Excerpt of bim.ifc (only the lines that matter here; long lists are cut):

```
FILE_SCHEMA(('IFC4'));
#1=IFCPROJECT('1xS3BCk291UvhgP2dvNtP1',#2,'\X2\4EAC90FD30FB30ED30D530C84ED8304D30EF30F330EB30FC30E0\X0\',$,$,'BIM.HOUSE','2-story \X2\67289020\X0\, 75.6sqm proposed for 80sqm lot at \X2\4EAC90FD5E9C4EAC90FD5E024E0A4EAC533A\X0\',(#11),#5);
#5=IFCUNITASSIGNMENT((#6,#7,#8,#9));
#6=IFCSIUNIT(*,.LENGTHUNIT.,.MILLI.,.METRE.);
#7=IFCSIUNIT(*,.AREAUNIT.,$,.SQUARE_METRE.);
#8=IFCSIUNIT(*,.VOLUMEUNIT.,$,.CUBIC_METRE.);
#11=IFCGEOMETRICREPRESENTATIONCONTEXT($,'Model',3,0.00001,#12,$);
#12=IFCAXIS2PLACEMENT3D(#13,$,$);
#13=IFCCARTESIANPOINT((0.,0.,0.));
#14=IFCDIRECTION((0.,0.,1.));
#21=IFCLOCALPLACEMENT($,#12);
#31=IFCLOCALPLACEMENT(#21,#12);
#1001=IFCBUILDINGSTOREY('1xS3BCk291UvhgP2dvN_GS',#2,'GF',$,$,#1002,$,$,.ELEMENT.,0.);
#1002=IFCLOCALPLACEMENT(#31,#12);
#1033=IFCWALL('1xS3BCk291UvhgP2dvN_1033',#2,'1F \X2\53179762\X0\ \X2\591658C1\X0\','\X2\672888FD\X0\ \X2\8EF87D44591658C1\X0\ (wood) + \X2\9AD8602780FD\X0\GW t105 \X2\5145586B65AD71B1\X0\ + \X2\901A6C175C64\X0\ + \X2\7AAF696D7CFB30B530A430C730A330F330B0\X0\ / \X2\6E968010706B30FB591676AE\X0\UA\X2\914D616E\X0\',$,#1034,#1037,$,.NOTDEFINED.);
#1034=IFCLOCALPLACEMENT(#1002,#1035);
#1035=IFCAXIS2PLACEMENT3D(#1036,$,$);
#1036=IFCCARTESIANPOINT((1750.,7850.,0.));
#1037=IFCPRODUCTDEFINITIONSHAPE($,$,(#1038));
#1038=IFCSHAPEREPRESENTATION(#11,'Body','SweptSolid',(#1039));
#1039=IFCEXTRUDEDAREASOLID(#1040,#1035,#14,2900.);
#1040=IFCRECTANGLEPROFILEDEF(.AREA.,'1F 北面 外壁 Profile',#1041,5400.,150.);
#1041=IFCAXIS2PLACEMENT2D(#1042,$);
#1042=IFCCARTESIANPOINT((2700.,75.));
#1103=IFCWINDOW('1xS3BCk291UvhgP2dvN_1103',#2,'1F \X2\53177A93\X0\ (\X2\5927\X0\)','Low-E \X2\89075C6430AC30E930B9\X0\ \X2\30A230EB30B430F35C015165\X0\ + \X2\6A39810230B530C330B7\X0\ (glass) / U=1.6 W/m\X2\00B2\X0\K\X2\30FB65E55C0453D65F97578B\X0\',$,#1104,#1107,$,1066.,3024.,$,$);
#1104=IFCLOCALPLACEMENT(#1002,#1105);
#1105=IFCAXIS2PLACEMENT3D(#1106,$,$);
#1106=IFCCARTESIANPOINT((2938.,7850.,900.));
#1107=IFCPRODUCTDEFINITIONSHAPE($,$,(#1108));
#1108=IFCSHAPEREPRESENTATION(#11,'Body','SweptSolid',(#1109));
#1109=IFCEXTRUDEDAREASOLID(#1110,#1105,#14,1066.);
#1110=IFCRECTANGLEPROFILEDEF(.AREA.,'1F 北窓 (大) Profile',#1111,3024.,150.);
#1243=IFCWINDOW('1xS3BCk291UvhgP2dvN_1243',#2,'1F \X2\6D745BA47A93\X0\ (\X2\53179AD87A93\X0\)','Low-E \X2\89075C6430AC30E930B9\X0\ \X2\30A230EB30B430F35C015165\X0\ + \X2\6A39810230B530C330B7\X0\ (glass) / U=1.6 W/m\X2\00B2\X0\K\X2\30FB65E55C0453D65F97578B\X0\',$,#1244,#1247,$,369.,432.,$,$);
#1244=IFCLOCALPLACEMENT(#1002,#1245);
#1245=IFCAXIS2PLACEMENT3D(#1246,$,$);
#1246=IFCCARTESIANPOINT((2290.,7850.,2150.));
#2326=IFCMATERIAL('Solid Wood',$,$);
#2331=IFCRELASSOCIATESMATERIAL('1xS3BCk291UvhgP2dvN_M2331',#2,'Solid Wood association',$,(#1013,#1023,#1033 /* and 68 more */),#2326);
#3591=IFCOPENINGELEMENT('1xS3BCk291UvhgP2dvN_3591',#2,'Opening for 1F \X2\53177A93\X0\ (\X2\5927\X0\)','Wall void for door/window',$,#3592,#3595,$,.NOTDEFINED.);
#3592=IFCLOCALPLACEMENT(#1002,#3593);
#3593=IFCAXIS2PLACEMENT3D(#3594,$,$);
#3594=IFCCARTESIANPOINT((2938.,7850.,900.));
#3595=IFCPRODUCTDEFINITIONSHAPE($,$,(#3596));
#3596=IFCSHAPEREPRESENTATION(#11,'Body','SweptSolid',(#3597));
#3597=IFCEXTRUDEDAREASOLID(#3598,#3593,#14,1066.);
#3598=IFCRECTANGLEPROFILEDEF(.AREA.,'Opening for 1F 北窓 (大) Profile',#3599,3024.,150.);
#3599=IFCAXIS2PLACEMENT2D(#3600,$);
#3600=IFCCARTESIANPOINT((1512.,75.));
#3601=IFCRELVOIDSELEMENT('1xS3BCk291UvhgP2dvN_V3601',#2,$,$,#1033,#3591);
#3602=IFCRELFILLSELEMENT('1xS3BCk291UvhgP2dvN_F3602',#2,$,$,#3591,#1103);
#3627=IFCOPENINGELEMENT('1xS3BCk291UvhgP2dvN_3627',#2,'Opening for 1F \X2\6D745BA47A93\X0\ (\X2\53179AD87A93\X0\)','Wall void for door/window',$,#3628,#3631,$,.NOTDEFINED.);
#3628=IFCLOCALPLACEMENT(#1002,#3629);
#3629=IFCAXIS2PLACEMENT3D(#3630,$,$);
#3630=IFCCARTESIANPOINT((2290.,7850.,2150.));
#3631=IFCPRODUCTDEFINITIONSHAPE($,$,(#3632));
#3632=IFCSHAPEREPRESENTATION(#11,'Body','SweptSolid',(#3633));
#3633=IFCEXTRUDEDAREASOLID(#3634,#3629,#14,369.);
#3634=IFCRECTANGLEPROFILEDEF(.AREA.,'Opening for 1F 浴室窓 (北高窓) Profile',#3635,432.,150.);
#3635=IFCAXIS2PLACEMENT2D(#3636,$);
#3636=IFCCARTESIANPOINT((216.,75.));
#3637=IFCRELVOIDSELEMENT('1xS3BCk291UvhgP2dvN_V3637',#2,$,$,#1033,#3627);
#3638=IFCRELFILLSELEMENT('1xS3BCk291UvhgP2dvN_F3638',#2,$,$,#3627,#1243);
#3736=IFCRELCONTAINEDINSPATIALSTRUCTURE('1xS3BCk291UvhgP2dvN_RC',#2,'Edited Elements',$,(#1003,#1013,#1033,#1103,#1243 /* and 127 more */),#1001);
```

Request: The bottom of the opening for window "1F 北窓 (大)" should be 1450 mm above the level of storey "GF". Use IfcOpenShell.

```python
import numpy as np
import ifcopenshell
import ifcopenshell.api.geometry
import ifcopenshell.geom
import ifcopenshell.util.element
import ifcopenshell.util.placement
import ifcopenshell.util.shape
import ifcopenshell.util.unit

model = ifcopenshell.open("bim.ifc")
unit_scale = ifcopenshell.util.unit.calculate_unit_scale(model)

window = model.by_guid("1xS3BCk291UvhgP2dvN_1103")
opening = window.FillsVoids[0].RelatingOpeningElement
storey = ifcopenshell.util.element.get_container(window, ifc_class="IfcBuildingStorey")
level = ifcopenshell.util.placement.get_local_placement(storey.ObjectPlacement)[2, 3]

# The opening's origin need not be at the sill, so measure its lowest point.
shape = ifcopenshell.geom.create_shape(ifcopenshell.geom.settings(), opening)
bottom = ifcopenshell.util.shape.get_shape_bottom_elevation(shape, shape.geometry) / unit_scale
dz = level + 1.45 / unit_scale - bottom

shift = np.array([0.0, 0.0, dz])
# The window is not placed relative to its opening, so move both.
for product in (opening, window):
    matrix = ifcopenshell.util.placement.get_local_placement(product.ObjectPlacement)
    matrix[:3, 3] += shift
    ifcopenshell.api.geometry.edit_object_placement(model, product=product, matrix=matrix, is_si=False)

print(f"moved by {dz * unit_scale:+.3f} m")

model.write("bim_v2.ifc")
```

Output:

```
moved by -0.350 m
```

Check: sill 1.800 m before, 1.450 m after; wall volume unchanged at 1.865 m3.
